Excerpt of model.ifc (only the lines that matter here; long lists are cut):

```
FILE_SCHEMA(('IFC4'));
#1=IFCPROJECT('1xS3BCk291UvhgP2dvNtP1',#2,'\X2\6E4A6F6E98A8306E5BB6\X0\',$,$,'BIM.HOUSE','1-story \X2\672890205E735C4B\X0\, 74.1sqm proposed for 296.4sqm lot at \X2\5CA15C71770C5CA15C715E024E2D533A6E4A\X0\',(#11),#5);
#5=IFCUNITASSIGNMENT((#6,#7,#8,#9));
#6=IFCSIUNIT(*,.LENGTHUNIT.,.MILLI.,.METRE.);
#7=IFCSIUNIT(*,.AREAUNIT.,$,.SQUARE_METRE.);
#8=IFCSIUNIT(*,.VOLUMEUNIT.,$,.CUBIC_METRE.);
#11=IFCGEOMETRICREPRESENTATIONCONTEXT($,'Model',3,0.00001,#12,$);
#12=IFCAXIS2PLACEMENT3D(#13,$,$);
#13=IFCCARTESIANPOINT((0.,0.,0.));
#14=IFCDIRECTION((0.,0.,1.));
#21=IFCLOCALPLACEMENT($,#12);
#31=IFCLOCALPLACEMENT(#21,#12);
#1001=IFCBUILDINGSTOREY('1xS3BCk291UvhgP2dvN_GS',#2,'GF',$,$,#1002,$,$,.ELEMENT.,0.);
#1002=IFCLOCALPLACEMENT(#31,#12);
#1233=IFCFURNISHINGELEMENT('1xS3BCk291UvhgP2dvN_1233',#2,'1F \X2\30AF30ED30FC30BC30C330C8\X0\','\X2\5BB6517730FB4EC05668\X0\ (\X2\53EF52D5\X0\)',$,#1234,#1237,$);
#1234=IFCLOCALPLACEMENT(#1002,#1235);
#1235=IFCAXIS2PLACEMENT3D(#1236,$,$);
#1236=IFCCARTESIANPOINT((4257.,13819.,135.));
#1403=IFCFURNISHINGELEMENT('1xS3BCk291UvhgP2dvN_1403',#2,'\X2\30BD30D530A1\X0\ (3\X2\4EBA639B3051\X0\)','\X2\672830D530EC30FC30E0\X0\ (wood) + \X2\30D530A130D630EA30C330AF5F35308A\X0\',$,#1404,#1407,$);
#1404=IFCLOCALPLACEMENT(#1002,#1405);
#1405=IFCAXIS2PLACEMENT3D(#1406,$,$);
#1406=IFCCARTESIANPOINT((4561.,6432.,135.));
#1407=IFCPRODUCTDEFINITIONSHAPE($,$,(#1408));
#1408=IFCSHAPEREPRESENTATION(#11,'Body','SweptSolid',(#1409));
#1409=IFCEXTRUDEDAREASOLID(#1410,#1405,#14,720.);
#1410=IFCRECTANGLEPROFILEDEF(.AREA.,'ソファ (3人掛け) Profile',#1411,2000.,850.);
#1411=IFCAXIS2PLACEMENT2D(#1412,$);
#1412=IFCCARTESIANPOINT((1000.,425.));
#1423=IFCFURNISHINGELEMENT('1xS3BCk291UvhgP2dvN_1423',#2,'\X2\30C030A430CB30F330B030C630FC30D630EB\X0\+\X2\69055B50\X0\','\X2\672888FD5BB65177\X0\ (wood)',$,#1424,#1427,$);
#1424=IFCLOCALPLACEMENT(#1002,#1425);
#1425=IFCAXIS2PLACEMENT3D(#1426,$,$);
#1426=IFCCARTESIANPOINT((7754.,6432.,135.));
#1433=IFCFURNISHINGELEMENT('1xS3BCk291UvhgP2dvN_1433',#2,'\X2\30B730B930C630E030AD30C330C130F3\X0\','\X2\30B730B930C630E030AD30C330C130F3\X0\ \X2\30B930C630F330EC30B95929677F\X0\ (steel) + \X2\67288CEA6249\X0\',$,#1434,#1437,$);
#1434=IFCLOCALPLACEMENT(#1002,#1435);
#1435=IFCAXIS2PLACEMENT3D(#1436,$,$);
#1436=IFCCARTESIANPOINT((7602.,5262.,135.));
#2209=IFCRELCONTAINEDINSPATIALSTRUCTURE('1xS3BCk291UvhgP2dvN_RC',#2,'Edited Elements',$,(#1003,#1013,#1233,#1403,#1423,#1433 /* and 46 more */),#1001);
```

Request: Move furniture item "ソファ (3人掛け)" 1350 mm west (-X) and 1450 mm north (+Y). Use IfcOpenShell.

```python
import ifcopenshell
import ifcopenshell.api.geometry
import ifcopenshell.util.placement
import ifcopenshell.util.unit

model = ifcopenshell.open("model.ifc")
unit_scale = ifcopenshell.util.unit.calculate_unit_scale(model)

item = model.by_guid("1xS3BCk291UvhgP2dvN_1403")
matrix = ifcopenshell.util.placement.get_local_placement(item.ObjectPlacement)
matrix[0, 3] -= 1.35 / unit_scale
matrix[1, 3] += 1.45 / unit_scale
ifcopenshell.api.geometry.edit_object_placement(model, product=item, matrix=matrix, is_si=False)

print(ifcopenshell.util.placement.get_local_placement(item.ObjectPlacement).round(3) + 0.0)

model.write("model_updated.ifc")
```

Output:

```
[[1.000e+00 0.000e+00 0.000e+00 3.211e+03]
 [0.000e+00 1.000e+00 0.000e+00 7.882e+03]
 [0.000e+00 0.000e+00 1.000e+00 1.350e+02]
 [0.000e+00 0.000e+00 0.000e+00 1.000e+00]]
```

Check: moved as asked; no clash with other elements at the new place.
